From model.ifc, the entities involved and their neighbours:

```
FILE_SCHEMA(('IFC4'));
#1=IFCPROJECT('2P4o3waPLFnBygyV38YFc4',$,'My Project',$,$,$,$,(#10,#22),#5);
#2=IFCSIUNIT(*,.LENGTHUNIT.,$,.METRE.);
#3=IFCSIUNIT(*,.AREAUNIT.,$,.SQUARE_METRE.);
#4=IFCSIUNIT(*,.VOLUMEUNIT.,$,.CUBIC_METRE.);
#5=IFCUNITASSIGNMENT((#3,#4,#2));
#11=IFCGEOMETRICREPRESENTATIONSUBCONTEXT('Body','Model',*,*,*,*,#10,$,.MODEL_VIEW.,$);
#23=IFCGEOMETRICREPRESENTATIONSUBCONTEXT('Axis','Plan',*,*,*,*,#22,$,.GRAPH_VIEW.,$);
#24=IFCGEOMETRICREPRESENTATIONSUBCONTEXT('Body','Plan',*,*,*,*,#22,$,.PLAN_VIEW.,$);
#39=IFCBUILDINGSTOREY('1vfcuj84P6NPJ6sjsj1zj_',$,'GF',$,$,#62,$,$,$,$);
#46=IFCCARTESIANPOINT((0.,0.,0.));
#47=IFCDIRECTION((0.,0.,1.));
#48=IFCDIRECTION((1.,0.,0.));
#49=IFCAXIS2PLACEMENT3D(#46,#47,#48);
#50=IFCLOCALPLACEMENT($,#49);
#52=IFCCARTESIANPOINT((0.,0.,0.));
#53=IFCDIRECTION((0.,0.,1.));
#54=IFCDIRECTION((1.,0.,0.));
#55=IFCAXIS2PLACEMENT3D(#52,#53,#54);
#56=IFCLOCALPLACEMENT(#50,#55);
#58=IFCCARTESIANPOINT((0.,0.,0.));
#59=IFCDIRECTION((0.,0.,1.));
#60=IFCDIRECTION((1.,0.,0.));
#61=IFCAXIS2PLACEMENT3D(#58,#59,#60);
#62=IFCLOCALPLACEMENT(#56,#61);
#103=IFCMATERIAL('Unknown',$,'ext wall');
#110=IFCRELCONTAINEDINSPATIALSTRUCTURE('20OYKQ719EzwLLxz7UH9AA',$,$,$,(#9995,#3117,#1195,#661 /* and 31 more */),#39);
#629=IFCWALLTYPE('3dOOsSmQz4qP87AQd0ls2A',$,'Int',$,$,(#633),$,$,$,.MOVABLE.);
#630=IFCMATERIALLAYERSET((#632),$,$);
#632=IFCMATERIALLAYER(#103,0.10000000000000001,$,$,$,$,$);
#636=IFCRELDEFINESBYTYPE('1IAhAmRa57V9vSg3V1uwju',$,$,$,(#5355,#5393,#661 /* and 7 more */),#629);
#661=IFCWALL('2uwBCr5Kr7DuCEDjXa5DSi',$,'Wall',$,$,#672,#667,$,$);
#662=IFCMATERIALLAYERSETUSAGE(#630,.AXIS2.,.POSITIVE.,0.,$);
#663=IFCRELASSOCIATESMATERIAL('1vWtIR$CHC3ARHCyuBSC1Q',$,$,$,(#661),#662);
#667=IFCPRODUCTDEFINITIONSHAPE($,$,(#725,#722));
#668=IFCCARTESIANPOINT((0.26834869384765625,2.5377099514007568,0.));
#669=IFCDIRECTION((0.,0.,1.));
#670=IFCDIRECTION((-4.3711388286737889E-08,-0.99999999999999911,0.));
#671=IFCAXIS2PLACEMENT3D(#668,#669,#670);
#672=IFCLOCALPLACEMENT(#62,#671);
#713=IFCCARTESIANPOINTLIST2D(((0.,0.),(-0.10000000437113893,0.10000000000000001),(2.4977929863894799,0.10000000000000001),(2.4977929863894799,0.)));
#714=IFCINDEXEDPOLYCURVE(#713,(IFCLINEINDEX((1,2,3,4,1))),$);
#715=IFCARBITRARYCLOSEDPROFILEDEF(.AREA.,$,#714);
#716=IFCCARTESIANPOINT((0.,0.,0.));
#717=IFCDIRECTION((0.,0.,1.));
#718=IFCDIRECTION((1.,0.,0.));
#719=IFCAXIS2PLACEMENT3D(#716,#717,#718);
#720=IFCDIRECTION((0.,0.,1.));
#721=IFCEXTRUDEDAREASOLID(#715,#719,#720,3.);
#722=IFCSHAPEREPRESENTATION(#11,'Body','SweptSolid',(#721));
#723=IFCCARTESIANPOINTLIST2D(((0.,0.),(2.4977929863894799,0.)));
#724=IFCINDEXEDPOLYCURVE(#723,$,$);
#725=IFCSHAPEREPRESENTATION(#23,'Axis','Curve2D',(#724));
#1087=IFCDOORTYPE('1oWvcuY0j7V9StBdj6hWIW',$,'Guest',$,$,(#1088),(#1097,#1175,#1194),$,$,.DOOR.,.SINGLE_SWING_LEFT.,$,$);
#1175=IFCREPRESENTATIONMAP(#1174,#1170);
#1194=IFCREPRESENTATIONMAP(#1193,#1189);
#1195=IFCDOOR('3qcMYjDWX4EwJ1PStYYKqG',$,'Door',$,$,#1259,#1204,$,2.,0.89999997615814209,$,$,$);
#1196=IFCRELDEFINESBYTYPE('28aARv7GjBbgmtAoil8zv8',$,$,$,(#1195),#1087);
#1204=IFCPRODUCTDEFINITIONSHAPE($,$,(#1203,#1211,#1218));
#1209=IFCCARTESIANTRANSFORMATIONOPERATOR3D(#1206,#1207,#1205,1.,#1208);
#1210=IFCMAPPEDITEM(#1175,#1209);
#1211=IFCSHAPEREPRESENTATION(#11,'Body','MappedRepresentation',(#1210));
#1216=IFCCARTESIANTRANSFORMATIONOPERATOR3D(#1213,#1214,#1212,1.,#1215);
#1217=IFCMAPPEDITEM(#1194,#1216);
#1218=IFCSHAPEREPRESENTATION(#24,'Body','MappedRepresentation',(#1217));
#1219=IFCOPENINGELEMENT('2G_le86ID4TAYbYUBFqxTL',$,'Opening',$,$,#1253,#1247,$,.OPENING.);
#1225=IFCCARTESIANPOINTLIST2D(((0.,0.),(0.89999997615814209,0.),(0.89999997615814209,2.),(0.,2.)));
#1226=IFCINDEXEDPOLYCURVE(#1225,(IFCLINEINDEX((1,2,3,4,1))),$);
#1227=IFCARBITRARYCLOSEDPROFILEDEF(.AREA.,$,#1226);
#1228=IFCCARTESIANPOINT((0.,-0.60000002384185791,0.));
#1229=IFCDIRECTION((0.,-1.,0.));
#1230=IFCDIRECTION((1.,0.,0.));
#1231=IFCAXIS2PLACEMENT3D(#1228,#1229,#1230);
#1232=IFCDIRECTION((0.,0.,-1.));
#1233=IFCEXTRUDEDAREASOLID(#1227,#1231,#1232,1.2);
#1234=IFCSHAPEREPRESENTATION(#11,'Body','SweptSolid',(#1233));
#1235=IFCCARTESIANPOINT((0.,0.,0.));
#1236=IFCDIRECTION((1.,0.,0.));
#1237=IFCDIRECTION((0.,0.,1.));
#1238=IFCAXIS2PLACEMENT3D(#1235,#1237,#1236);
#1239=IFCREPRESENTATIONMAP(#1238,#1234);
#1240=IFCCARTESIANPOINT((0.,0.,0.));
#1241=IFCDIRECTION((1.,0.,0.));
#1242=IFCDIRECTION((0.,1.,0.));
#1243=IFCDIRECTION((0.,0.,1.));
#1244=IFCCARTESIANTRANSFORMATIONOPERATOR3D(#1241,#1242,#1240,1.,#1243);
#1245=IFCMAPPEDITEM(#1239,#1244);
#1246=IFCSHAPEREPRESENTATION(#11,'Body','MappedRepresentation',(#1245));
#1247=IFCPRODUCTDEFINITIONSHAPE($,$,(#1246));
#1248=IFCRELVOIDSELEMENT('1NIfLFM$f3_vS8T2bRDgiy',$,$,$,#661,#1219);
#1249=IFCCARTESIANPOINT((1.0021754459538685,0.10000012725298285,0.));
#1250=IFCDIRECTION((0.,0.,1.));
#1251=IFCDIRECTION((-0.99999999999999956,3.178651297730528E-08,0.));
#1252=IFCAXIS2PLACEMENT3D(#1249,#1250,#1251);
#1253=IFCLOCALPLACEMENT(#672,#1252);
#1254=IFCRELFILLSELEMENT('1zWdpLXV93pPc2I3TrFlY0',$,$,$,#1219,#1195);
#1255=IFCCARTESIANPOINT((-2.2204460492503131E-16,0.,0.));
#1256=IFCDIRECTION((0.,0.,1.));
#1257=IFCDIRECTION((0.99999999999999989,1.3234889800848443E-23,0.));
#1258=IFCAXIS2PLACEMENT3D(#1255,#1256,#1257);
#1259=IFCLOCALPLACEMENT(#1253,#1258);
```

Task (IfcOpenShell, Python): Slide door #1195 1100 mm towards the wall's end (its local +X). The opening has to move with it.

```python
import ifcopenshell
import ifcopenshell.api.geometry
import ifcopenshell.util.placement
import ifcopenshell.util.unit

model = ifcopenshell.open("model.ifc")
unit_scale = ifcopenshell.util.unit.calculate_unit_scale(model)

door = model.by_guid("3qcMYjDWX4EwJ1PStYYKqG")
opening = door.FillsVoids[0].RelatingOpeningElement
wall = opening.VoidsElements[0].RelatingBuildingElement

wall_matrix = ifcopenshell.util.placement.get_local_placement(wall.ObjectPlacement)
shift = wall_matrix[:3, 0] * 1.1 / unit_scale
before = ifcopenshell.util.placement.get_local_placement(door.ObjectPlacement)[:3, 3].copy()

# The door is placed relative to its opening, so it follows when the opening moves.
matrix = ifcopenshell.util.placement.get_local_placement(opening.ObjectPlacement)
matrix[:3, 3] += shift
ifcopenshell.api.geometry.edit_object_placement(
    model, product=opening, matrix=matrix, is_si=False, should_transform_children=True
)

after = ifcopenshell.util.placement.get_local_placement(door.ObjectPlacement)[:3, 3]
print("door moved by", (after - before).round(3) + 0.0)

model.write("model_v2.ifc")
```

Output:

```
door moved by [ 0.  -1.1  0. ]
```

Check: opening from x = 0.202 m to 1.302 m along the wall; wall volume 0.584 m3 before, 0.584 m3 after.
